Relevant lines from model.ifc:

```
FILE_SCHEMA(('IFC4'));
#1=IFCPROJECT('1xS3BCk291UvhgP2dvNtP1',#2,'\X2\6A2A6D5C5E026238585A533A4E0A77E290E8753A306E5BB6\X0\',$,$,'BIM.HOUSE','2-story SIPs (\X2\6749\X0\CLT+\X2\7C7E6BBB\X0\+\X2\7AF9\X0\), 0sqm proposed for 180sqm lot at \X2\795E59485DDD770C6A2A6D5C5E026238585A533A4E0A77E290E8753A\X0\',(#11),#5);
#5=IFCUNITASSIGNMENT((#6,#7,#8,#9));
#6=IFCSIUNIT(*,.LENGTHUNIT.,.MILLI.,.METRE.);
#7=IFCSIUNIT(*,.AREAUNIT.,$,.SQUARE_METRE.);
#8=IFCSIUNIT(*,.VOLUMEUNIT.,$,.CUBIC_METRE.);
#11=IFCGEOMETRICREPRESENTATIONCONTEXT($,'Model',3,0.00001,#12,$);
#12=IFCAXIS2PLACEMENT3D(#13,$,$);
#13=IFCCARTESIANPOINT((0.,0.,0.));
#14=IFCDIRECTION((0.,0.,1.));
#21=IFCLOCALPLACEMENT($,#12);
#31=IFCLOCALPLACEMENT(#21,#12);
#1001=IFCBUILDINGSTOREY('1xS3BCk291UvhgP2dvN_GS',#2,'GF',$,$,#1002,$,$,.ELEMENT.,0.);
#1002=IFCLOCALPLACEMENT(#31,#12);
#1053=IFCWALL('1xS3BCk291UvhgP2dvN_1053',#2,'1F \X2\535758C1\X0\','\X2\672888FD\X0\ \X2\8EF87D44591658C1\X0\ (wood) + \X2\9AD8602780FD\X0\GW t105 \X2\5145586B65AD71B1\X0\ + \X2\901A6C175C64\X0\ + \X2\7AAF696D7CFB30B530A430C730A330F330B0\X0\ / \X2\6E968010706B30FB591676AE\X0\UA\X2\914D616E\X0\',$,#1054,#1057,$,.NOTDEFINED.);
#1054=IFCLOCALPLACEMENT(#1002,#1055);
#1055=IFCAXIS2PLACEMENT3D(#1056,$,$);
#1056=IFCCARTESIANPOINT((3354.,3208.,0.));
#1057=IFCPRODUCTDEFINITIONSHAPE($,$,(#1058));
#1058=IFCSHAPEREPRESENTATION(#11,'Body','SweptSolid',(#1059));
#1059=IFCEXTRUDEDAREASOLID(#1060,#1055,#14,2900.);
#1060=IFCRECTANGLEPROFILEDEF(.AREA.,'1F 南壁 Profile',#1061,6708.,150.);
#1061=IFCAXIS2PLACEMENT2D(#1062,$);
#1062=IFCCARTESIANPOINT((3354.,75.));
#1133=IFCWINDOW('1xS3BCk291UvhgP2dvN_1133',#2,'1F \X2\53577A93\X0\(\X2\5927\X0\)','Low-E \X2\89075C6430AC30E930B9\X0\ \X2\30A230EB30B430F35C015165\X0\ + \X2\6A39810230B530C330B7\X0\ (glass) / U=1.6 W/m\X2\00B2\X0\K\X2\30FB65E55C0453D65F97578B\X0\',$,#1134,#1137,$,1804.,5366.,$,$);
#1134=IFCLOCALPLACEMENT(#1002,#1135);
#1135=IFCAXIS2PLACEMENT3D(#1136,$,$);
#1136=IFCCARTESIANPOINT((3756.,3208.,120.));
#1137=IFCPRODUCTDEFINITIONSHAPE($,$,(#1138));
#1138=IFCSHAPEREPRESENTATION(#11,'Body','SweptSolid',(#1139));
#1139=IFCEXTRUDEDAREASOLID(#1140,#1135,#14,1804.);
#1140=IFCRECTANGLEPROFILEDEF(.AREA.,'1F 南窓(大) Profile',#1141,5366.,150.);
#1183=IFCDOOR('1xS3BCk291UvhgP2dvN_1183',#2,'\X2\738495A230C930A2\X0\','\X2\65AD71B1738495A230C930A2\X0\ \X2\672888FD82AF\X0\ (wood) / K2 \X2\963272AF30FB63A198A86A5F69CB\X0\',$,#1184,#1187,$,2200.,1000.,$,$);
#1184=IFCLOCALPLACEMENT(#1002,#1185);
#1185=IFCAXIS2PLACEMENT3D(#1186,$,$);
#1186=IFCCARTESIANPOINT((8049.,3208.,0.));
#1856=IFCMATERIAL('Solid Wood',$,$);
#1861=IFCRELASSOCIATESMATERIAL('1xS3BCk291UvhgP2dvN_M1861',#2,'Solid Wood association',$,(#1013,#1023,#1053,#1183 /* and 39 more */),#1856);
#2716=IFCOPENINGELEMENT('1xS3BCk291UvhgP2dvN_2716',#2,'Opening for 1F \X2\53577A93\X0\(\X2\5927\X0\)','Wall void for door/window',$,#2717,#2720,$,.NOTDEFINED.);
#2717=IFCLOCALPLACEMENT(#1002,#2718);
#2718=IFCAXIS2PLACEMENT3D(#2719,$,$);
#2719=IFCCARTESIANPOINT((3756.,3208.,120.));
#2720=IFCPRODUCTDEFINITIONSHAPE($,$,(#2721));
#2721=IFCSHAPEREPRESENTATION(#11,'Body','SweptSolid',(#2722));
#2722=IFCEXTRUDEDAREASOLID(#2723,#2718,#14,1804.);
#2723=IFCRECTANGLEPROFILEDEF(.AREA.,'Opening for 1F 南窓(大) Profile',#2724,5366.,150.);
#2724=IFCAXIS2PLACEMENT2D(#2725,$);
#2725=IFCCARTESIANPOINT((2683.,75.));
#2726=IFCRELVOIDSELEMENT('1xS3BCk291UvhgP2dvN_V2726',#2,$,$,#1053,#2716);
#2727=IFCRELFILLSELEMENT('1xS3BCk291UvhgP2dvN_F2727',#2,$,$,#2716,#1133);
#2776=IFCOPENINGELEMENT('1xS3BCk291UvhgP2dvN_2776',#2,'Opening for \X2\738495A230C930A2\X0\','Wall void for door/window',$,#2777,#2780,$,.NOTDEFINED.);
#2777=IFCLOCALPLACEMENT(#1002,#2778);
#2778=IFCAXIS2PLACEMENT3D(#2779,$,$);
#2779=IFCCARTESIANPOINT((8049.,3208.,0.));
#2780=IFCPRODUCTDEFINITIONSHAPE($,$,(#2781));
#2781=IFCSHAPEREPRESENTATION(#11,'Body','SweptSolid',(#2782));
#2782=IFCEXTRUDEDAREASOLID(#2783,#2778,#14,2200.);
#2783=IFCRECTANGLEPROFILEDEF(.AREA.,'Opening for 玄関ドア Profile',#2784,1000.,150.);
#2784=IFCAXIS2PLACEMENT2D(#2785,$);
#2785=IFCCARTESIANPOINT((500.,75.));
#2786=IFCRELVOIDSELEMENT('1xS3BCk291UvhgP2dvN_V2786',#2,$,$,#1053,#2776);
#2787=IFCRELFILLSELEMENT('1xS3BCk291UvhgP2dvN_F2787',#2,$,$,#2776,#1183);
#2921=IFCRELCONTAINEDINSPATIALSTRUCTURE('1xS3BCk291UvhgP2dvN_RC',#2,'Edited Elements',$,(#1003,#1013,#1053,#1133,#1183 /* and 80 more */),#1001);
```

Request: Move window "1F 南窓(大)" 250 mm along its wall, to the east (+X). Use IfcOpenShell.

```python
import ifcopenshell
import ifcopenshell.api.geometry
import ifcopenshell.util.placement
import ifcopenshell.util.unit

model = ifcopenshell.open("model.ifc")
unit_scale = ifcopenshell.util.unit.calculate_unit_scale(model)

window = model.by_guid("1xS3BCk291UvhgP2dvN_1133")
opening = window.FillsVoids[0].RelatingOpeningElement
wall = opening.VoidsElements[0].RelatingBuildingElement

wall_matrix = ifcopenshell.util.placement.get_local_placement(wall.ObjectPlacement)
shift = wall_matrix[:3, 0] * 0.25 / unit_scale
before = ifcopenshell.util.placement.get_local_placement(window.ObjectPlacement)[:3, 3].copy()

# The window is not placed relative to its opening, so move both.
for product in (opening, window):
    matrix = ifcopenshell.util.placement.get_local_placement(product.ObjectPlacement)
    matrix[:3, 3] += shift
    ifcopenshell.api.geometry.edit_object_placement(model, product=product, matrix=matrix, is_si=False)

after = ifcopenshell.util.placement.get_local_placement(window.ObjectPlacement)[:3, 3]
print("window moved by", (after - before).round(3) + 0.0)

model.write("model_rev.ifc")
```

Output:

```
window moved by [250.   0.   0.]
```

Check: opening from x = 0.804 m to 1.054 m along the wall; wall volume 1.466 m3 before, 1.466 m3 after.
